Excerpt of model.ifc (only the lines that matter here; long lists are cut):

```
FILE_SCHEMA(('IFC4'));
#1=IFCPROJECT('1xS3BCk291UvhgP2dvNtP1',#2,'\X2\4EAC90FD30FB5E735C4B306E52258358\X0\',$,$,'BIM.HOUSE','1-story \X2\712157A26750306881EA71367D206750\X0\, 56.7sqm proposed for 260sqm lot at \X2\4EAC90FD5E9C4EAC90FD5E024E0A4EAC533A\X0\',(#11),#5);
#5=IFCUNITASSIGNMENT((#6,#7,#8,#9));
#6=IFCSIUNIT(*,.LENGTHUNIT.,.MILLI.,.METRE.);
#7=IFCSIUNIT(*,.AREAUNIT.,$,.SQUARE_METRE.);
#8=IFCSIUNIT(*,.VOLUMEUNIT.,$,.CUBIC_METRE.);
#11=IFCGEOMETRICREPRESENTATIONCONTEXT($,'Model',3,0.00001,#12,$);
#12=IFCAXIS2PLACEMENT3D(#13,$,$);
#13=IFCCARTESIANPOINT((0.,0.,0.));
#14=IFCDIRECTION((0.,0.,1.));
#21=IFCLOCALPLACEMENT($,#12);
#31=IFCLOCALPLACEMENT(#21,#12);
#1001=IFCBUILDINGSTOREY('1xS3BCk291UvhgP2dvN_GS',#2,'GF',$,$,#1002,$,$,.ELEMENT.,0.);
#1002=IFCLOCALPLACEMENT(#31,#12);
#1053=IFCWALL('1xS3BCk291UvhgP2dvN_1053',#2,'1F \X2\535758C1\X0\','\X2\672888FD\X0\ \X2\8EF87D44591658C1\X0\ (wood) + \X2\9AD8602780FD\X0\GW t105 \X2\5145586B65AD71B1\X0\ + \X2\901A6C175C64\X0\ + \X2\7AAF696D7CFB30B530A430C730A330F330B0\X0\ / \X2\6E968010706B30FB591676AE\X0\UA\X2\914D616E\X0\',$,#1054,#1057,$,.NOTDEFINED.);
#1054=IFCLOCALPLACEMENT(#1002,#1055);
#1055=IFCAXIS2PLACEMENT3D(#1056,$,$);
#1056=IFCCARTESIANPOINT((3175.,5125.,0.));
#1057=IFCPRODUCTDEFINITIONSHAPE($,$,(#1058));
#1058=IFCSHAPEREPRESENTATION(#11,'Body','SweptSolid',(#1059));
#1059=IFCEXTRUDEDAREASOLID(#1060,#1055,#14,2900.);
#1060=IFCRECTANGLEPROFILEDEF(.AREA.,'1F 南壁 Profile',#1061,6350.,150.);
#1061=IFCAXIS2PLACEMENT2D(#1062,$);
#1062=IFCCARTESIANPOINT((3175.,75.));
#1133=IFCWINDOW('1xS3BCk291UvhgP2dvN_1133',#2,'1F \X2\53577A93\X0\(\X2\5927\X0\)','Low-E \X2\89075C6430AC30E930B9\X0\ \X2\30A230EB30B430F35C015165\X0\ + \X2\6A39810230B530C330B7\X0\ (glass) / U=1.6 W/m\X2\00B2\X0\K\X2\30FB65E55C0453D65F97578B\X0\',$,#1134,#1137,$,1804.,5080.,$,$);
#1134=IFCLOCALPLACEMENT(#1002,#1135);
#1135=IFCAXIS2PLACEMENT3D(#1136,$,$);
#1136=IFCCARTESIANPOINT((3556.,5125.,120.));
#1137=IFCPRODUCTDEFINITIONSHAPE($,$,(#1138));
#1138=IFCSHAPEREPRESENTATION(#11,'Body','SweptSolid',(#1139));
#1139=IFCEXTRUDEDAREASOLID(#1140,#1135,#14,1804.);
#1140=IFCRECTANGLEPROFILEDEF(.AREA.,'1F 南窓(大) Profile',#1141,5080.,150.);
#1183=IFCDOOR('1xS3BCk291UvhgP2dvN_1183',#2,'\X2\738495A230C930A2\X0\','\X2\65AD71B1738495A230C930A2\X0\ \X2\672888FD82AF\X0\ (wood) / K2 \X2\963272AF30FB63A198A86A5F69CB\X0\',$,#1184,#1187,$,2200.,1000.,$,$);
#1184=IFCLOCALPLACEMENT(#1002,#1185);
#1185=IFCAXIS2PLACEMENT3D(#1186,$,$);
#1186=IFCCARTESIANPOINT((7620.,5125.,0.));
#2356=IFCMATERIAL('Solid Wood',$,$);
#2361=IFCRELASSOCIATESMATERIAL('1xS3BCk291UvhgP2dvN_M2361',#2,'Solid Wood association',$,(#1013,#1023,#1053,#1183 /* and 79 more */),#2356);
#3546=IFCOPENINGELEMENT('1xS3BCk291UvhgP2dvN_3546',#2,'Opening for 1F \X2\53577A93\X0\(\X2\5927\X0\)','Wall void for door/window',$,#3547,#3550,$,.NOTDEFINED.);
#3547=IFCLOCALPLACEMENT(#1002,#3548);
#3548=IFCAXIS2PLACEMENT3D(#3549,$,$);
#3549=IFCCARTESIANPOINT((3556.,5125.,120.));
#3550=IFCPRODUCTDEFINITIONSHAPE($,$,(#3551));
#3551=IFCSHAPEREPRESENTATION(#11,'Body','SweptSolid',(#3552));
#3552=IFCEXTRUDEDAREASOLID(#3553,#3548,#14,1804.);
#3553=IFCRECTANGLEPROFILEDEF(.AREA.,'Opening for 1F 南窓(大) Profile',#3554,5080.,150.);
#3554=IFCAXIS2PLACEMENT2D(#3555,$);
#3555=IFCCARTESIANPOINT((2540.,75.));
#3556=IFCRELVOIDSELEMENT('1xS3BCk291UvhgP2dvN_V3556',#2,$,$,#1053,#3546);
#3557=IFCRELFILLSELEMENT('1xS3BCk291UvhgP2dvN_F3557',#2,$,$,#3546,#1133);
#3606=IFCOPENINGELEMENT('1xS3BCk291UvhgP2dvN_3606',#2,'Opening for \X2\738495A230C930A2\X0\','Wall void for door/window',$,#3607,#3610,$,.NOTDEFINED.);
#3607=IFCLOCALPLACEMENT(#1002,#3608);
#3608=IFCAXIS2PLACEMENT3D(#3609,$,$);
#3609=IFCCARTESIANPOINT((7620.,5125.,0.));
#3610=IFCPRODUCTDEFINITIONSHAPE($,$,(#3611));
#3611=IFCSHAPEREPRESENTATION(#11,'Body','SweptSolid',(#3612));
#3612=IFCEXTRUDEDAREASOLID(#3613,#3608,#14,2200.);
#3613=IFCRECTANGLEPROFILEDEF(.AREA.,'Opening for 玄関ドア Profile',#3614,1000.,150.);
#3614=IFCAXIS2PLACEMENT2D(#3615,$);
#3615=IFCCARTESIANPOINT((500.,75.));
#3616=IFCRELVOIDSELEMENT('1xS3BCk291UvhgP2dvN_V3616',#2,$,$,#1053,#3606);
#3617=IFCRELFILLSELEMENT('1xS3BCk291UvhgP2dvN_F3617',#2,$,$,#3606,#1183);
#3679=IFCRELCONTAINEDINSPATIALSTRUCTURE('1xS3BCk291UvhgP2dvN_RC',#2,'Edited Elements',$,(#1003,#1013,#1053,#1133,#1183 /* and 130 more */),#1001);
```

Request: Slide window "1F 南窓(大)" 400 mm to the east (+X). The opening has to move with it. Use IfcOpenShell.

```python
import ifcopenshell
import ifcopenshell.api.geometry
import ifcopenshell.util.placement
import ifcopenshell.util.unit

model = ifcopenshell.open("model.ifc")
unit_scale = ifcopenshell.util.unit.calculate_unit_scale(model)

window = model.by_guid("1xS3BCk291UvhgP2dvN_1133")
opening = window.FillsVoids[0].RelatingOpeningElement
wall = opening.VoidsElements[0].RelatingBuildingElement

wall_matrix = ifcopenshell.util.placement.get_local_placement(wall.ObjectPlacement)
shift = wall_matrix[:3, 0] * 0.4 / unit_scale
before = ifcopenshell.util.placement.get_local_placement(window.ObjectPlacement)[:3, 3].copy()

# The window is not placed relative to its opening, so move both.
for product in (opening, window):
    matrix = ifcopenshell.util.placement.get_local_placement(product.ObjectPlacement)
    matrix[:3, 3] += shift
    ifcopenshell.api.geometry.edit_object_placement(model, product=product, matrix=matrix, is_si=False)

after = ifcopenshell.util.placement.get_local_placement(window.ObjectPlacement)[:3, 3]
print("window moved by", (after - before).round(3) + 0.0)

model.write("model_edited.ifc")
```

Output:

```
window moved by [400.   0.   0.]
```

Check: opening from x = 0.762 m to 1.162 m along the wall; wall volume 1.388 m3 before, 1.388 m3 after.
